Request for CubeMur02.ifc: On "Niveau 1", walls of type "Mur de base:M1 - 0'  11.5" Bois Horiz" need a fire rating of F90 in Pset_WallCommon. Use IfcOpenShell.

First a look at what the model holds.

```python
import ifcopenshell
import ifcopenshell.util.element

model = ifcopenshell.open("CubeMur02.ifc")
print(model.schema)
storey = next(s for s in model.by_type("IfcBuildingStorey") if s.Name == "Niveau 1")
walls = [e for e in ifcopenshell.util.element.get_decomposition(storey) if e.is_a("IfcWall")]
seen = {}
for e in walls:
    element_type = ifcopenshell.util.element.get_type(e)
    key = (element_type.Name if element_type != e and element_type else None, ifcopenshell.util.element.get_pset(e, "Pset_WallCommon", "FireRating"))
    seen[key] = seen.get(key, 0) + 1
for (name, value), count in sorted(seen.items(), key=str):
    print(count, "x", name, "|", value)
```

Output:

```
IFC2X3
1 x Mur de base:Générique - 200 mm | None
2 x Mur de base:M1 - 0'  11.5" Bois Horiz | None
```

```python
import ifcopenshell
import ifcopenshell.api.pset
import ifcopenshell.util.element

model = ifcopenshell.open("CubeMur02.ifc")

storey = next(s for s in model.by_type("IfcBuildingStorey") if s.Name == "Niveau 1")
walls = [e for e in ifcopenshell.util.element.get_decomposition(storey) if e.is_a("IfcWall")]

count = 0
for e in walls:
    element_type = ifcopenshell.util.element.get_type(e)
    if element_type in (None, e) or element_type.Name != 'Mur de base:M1 - 0\'  11.5" Bois Horiz':
        continue
    # add_pset returns the element's existing set when there is one.
    pset = ifcopenshell.api.pset.add_pset(model, product=e, name="Pset_WallCommon")
    ifcopenshell.api.pset.edit_pset(model, pset=pset, properties={"FireRating": "F90"})
    count += 1

print(count, "walls updated")

model.write("CubeMur02_rev.ifc")
```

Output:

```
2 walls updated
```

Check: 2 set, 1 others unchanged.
